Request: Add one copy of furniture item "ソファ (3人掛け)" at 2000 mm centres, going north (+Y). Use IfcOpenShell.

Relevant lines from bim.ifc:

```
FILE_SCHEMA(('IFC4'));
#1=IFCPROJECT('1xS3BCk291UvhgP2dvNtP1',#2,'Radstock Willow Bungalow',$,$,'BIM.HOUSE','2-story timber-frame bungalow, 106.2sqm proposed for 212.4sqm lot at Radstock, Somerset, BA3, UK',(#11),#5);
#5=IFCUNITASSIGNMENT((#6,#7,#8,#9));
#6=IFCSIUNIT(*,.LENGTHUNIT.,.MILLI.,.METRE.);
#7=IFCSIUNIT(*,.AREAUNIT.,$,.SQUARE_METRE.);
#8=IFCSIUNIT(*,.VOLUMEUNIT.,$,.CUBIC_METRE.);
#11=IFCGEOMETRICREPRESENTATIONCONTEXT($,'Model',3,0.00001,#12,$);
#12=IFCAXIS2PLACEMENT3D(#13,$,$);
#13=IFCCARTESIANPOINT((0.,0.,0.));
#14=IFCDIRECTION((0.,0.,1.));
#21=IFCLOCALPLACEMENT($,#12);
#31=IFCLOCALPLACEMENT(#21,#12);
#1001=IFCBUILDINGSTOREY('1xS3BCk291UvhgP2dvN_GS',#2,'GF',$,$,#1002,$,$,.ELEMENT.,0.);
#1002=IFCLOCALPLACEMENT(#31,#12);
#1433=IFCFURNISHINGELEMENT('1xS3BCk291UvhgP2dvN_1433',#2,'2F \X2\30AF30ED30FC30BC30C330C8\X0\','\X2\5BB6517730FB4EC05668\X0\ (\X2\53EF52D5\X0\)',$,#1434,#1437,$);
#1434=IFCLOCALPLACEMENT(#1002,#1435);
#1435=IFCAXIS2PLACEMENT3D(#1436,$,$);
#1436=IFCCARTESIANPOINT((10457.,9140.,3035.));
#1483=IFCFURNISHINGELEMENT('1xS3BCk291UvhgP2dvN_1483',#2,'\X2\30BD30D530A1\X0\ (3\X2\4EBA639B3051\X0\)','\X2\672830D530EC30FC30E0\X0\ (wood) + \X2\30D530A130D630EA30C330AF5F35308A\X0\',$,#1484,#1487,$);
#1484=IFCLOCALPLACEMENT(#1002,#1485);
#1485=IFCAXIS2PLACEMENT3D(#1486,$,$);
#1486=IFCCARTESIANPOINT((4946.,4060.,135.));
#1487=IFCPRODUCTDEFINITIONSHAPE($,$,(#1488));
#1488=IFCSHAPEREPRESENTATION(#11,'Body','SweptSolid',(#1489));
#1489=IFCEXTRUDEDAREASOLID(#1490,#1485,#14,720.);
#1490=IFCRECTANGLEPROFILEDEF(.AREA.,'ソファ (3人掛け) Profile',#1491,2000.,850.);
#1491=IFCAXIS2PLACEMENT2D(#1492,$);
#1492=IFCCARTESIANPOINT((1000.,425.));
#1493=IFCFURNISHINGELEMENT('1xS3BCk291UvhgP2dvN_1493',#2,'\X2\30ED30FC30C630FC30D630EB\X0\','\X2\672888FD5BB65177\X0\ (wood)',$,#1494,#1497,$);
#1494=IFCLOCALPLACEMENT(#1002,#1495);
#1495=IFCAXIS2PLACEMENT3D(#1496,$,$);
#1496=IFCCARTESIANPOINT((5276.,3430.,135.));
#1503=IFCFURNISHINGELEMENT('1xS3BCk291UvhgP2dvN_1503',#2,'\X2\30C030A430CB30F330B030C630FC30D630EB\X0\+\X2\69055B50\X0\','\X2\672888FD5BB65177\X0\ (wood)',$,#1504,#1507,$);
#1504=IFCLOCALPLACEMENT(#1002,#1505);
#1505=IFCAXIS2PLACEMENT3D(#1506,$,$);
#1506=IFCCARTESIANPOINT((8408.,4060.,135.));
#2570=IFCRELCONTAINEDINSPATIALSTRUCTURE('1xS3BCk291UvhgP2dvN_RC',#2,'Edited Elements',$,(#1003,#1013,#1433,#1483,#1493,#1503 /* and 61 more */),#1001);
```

```python
import numpy as np
import ifcopenshell
import ifcopenshell.api.geometry
import ifcopenshell.api.root
import ifcopenshell.util.element
import ifcopenshell.util.placement
import ifcopenshell.util.unit

model = ifcopenshell.open("bim.ifc")
unit_scale = ifcopenshell.util.unit.calculate_unit_scale(model)


def reuse_history(source, copy):
    """copy_class also copies each property set's owner history, people and application; keep the originals."""
    for rel in copy.IsDefinedBy:
        if rel.is_a("IfcRelDefinesByProperties") and (history := rel.RelatingPropertyDefinition.OwnerHistory):
            rel.RelatingPropertyDefinition.OwnerHistory = source.OwnerHistory
            ifcopenshell.util.element.remove_deep2(model, history)


source = model.by_id(1483)
base = ifcopenshell.util.placement.get_local_placement(source.ObjectPlacement)
step = np.array([0.0, 1.0, 0.0]) * 2 / unit_scale

for i in range(1, 2):
    copy = ifcopenshell.api.root.copy_class(model, product=source)
    copy.Representation = ifcopenshell.util.element.copy_deep(
        model, source.Representation, exclude=["IfcGeometricRepresentationContext", "IfcRepresentationMap"]
    )
    reuse_history(source, copy)
    matrix = base.copy()
    matrix[:3, 3] += i * step
    print("added at", matrix[:3, 3].round(3) + 0.0)
    ifcopenshell.api.geometry.edit_object_placement(model, product=copy, matrix=matrix, is_si=False)

model.write("bim_rev.ifc")
```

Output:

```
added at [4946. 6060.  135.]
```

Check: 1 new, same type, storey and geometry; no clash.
